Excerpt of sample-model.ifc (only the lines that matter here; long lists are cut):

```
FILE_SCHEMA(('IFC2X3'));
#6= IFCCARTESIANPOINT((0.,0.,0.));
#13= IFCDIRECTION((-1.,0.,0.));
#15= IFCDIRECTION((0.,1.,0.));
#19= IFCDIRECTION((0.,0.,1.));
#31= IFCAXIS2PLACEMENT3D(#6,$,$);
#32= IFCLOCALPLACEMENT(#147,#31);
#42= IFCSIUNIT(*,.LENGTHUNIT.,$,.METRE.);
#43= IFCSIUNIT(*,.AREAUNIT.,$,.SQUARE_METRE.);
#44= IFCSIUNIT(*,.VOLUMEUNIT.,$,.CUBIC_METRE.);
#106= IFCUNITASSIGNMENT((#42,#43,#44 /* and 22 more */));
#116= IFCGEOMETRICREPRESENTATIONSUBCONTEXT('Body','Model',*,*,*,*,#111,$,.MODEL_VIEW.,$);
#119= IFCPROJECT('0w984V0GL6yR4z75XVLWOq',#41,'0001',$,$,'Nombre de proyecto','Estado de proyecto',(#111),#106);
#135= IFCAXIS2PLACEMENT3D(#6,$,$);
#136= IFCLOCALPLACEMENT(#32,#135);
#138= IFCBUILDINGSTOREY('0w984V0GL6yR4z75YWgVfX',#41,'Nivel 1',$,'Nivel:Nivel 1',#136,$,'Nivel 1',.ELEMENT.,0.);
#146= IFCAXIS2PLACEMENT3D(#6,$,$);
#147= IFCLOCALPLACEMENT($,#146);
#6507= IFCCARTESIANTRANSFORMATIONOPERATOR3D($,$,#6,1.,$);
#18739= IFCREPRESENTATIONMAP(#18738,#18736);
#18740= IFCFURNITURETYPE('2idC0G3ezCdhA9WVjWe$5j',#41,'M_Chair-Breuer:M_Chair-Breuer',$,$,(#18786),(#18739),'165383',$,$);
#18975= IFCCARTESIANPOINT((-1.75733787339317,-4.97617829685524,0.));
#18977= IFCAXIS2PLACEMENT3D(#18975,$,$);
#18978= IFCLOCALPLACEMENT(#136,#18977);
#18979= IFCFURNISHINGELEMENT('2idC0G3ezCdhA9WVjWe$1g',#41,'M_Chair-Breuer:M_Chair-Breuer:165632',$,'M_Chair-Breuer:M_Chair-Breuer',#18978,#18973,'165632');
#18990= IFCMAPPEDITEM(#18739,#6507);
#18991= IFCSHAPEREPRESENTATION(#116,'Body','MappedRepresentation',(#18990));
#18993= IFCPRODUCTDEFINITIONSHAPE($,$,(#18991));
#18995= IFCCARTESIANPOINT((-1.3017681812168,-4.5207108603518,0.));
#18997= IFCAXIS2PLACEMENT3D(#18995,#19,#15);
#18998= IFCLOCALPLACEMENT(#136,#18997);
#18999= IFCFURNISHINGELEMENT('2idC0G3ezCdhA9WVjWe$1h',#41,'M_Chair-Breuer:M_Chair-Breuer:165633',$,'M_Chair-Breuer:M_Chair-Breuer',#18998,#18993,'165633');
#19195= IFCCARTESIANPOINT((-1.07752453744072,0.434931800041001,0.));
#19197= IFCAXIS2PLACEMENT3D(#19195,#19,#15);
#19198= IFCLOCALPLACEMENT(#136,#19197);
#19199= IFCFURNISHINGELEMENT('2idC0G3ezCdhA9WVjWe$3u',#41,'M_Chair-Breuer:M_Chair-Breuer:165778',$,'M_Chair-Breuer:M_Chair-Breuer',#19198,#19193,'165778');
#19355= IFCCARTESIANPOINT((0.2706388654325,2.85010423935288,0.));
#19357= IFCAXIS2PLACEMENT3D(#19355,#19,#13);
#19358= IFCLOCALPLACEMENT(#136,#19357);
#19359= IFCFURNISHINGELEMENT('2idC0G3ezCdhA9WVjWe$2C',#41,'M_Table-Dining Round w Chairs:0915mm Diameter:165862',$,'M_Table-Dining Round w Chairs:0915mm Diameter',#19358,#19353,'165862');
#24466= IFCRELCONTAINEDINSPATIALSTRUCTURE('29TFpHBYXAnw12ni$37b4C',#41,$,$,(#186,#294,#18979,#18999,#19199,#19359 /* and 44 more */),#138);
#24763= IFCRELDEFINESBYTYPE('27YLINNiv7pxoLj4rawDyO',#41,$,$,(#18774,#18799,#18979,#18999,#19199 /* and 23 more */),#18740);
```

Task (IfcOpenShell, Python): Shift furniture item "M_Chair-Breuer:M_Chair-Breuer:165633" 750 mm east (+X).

```python
import ifcopenshell
import ifcopenshell.api.geometry
import ifcopenshell.util.placement
import ifcopenshell.util.unit

model = ifcopenshell.open("sample-model.ifc")
unit_scale = ifcopenshell.util.unit.calculate_unit_scale(model)

item = model.by_guid("2idC0G3ezCdhA9WVjWe$1h")
matrix = ifcopenshell.util.placement.get_local_placement(item.ObjectPlacement)
matrix[0, 3] += 0.75 / unit_scale
ifcopenshell.api.geometry.edit_object_placement(model, product=item, matrix=matrix, is_si=False)

print(ifcopenshell.util.placement.get_local_placement(item.ObjectPlacement).round(3) + 0.0)

model.write("sample-model_rev.ifc")
```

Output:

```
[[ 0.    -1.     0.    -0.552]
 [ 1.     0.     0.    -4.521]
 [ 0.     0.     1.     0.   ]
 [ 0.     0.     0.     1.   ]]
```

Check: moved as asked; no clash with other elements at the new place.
